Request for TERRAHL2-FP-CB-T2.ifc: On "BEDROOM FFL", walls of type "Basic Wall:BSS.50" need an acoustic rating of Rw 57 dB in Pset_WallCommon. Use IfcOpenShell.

First a look at what the model holds.

```python
import ifcopenshell
import ifcopenshell.util.element

model = ifcopenshell.open("TERRAHL2-FP-CB-T2.ifc")
print(model.schema)
storey = next(s for s in model.by_type("IfcBuildingStorey") if s.Name == "BEDROOM FFL")
walls = [e for e in ifcopenshell.util.element.get_decomposition(storey) if e.is_a("IfcWall")]
seen = {}
for e in walls:
    element_type = ifcopenshell.util.element.get_type(e)
    key = (element_type.Name if element_type != e and element_type else None, ifcopenshell.util.element.get_pset(e, "Pset_WallCommon", "AcousticRating"))
    seen[key] = seen.get(key, 0) + 1
for (name, value), count in sorted(seen.items(), key=str):
    print(count, "x", name, "|", value)
```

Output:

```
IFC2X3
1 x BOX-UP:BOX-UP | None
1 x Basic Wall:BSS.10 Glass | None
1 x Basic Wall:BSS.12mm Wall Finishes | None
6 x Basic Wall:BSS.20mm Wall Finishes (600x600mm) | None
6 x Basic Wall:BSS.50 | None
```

```python
import ifcopenshell
import ifcopenshell.api.pset
import ifcopenshell.util.element

model = ifcopenshell.open("TERRAHL2-FP-CB-T2.ifc")

storey = next(s for s in model.by_type("IfcBuildingStorey") if s.Name == "BEDROOM FFL")
walls = [e for e in ifcopenshell.util.element.get_decomposition(storey) if e.is_a("IfcWall")]

count = 0
for e in walls:
    element_type = ifcopenshell.util.element.get_type(e)
    if element_type in (None, e) or element_type.Name != "Basic Wall:BSS.50":
        continue
    # add_pset returns the element's existing set when there is one.
    pset = ifcopenshell.api.pset.add_pset(model, product=e, name="Pset_WallCommon")
    ifcopenshell.api.pset.edit_pset(model, pset=pset, properties={"AcousticRating": "Rw 57 dB"})
    count += 1

print(count, "walls updated")

model.write("TERRAHL2-FP-CB-T2_rev.ifc")
```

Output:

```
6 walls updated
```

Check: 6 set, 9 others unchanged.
